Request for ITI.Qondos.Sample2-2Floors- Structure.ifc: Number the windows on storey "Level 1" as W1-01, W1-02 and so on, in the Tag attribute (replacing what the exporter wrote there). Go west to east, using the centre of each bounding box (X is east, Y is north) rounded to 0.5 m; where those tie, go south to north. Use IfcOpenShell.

First a look at what the model holds.

```python
import ifcopenshell
import ifcopenshell.util.element
import ifcopenshell.util.placement

model = ifcopenshell.open("ITI.Qondos.Sample2-2Floors- Structure.ifc")
print(model.schema)
storey = next(s for s in model.by_type("IfcBuildingStorey") if s.Name == "Level 1")
windows = [e for e in ifcopenshell.util.element.get_decomposition(storey) if e.is_a("IfcWindow")]
for e in sorted(windows, key=lambda e: e.id()):
    origin = ifcopenshell.util.placement.get_local_placement(e.ObjectPlacement)[:3, 3]
    print(e.id(), e.Tag, e.Name, origin.round(2) + 0.0, sep=" | ")
```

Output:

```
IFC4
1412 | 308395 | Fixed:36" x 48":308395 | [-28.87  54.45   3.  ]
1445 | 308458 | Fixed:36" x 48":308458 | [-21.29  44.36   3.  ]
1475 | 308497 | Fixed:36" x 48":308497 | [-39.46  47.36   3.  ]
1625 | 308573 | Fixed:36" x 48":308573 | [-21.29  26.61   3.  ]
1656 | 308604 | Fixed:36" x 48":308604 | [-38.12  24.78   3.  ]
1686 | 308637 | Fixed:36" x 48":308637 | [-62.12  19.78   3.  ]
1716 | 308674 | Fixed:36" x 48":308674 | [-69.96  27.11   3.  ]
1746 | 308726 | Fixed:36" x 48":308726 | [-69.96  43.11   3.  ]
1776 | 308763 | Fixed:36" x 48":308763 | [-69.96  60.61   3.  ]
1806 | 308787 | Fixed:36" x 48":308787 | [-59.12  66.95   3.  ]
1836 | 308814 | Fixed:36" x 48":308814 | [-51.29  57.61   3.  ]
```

```python
import ifcopenshell
import ifcopenshell.geom
import ifcopenshell.util.element
import ifcopenshell.util.shape

model = ifcopenshell.open("ITI.Qondos.Sample2-2Floors- Structure.ifc")
settings = ifcopenshell.geom.settings()
settings.set("use-world-coords", True)


def centre(element):
    shape = ifcopenshell.geom.create_shape(settings, element)
    return ifcopenshell.util.shape.get_bbox_centroid(shape.geometry)


storey = next(s for s in model.by_type("IfcBuildingStorey") if s.Name == "Level 1")
windows = [e for e in ifcopenshell.util.element.get_decomposition(storey) if e.is_a("IfcWindow")]

# Insertion points can sit at a corner or the storey origin, so sort by the geometry (in metres).
centres = {e: centre(e) for e in windows}
windows.sort(key=lambda e: (round(centres[e][0] / 0.5), centres[e][1]))

for i, e in enumerate(windows, start=1):
    number = f"W1-{i:02d}"
    e.Tag = number
    print(e.id(), number)

model.write("ITI.Qondos.Sample2-2Floors- Structure_updated.ifc")
```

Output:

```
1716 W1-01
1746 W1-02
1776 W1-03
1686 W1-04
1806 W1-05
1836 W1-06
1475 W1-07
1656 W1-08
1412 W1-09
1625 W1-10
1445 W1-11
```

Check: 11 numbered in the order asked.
